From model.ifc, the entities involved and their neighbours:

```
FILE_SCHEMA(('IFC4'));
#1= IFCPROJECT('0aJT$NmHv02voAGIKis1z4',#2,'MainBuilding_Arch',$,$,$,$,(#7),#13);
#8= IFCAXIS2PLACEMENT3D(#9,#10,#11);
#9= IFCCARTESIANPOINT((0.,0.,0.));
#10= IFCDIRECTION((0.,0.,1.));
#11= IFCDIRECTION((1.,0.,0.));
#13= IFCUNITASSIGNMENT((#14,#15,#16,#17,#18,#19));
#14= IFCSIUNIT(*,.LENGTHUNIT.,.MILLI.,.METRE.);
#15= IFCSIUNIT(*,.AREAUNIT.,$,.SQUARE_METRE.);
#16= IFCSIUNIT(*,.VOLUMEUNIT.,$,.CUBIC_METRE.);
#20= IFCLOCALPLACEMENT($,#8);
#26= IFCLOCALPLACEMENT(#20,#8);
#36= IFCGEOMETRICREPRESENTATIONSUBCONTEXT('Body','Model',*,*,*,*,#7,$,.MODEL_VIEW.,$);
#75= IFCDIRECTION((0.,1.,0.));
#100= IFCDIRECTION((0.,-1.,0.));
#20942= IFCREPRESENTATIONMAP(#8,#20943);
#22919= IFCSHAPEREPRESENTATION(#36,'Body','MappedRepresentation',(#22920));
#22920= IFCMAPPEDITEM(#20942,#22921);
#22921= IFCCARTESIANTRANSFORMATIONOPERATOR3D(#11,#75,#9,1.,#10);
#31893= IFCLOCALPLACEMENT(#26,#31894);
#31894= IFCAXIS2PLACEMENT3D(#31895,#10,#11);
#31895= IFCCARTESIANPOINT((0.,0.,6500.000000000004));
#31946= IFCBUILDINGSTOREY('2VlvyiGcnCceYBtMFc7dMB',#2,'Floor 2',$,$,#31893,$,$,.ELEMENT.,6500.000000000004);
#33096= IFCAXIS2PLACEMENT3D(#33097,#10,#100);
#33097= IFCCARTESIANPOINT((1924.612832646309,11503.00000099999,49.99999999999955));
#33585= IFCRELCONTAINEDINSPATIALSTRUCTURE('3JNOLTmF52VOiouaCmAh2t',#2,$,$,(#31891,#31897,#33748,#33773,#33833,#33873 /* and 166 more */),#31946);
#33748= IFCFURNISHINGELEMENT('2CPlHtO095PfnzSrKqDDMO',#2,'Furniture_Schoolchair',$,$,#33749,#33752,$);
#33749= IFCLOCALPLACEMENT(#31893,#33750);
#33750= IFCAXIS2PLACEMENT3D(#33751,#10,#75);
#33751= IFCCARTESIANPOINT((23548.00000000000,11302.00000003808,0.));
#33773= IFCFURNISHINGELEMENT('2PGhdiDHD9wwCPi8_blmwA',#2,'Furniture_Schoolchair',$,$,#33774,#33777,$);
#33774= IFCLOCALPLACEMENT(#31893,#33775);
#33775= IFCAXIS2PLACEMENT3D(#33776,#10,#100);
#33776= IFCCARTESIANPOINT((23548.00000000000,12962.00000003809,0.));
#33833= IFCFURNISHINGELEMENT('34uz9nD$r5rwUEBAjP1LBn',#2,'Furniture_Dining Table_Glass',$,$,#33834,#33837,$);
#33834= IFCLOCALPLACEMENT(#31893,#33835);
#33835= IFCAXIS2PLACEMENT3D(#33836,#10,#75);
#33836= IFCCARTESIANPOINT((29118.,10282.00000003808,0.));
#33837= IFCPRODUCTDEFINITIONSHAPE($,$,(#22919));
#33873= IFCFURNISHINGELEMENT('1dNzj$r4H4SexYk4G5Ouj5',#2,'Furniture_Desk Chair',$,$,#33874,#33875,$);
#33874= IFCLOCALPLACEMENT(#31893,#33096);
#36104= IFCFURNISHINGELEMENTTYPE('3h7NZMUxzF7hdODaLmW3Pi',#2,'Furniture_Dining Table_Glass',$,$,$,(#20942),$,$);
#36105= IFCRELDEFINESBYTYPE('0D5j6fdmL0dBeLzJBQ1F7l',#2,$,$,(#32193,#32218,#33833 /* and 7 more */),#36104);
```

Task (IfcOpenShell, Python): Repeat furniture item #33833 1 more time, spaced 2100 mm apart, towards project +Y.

```python
import numpy as np
import ifcopenshell
import ifcopenshell.api.geometry
import ifcopenshell.api.root
import ifcopenshell.util.element
import ifcopenshell.util.placement
import ifcopenshell.util.unit

model = ifcopenshell.open("model.ifc")
unit_scale = ifcopenshell.util.unit.calculate_unit_scale(model)


def reuse_history(source, copy):
    """copy_class also copies each property set's owner history, people and application; keep the originals."""
    for rel in copy.IsDefinedBy:
        if rel.is_a("IfcRelDefinesByProperties") and (history := rel.RelatingPropertyDefinition.OwnerHistory):
            rel.RelatingPropertyDefinition.OwnerHistory = source.OwnerHistory
            ifcopenshell.util.element.remove_deep2(model, history)


source = model.by_guid("34uz9nD$r5rwUEBAjP1LBn")
base = ifcopenshell.util.placement.get_local_placement(source.ObjectPlacement)
step = np.array([0.0, 1.0, 0.0]) * 2.1 / unit_scale

for i in range(1, 2):
    copy = ifcopenshell.api.root.copy_class(model, product=source)
    copy.Representation = ifcopenshell.util.element.copy_deep(
        model, source.Representation, exclude=["IfcGeometricRepresentationContext", "IfcRepresentationMap"]
    )
    reuse_history(source, copy)
    matrix = base.copy()
    matrix[:3, 3] += i * step
    print("added at", matrix[:3, 3].round(3) + 0.0)
    ifcopenshell.api.geometry.edit_object_placement(model, product=copy, matrix=matrix, is_si=False)

model.write("model_updated.ifc")
```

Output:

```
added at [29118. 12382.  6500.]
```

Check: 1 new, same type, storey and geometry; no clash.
